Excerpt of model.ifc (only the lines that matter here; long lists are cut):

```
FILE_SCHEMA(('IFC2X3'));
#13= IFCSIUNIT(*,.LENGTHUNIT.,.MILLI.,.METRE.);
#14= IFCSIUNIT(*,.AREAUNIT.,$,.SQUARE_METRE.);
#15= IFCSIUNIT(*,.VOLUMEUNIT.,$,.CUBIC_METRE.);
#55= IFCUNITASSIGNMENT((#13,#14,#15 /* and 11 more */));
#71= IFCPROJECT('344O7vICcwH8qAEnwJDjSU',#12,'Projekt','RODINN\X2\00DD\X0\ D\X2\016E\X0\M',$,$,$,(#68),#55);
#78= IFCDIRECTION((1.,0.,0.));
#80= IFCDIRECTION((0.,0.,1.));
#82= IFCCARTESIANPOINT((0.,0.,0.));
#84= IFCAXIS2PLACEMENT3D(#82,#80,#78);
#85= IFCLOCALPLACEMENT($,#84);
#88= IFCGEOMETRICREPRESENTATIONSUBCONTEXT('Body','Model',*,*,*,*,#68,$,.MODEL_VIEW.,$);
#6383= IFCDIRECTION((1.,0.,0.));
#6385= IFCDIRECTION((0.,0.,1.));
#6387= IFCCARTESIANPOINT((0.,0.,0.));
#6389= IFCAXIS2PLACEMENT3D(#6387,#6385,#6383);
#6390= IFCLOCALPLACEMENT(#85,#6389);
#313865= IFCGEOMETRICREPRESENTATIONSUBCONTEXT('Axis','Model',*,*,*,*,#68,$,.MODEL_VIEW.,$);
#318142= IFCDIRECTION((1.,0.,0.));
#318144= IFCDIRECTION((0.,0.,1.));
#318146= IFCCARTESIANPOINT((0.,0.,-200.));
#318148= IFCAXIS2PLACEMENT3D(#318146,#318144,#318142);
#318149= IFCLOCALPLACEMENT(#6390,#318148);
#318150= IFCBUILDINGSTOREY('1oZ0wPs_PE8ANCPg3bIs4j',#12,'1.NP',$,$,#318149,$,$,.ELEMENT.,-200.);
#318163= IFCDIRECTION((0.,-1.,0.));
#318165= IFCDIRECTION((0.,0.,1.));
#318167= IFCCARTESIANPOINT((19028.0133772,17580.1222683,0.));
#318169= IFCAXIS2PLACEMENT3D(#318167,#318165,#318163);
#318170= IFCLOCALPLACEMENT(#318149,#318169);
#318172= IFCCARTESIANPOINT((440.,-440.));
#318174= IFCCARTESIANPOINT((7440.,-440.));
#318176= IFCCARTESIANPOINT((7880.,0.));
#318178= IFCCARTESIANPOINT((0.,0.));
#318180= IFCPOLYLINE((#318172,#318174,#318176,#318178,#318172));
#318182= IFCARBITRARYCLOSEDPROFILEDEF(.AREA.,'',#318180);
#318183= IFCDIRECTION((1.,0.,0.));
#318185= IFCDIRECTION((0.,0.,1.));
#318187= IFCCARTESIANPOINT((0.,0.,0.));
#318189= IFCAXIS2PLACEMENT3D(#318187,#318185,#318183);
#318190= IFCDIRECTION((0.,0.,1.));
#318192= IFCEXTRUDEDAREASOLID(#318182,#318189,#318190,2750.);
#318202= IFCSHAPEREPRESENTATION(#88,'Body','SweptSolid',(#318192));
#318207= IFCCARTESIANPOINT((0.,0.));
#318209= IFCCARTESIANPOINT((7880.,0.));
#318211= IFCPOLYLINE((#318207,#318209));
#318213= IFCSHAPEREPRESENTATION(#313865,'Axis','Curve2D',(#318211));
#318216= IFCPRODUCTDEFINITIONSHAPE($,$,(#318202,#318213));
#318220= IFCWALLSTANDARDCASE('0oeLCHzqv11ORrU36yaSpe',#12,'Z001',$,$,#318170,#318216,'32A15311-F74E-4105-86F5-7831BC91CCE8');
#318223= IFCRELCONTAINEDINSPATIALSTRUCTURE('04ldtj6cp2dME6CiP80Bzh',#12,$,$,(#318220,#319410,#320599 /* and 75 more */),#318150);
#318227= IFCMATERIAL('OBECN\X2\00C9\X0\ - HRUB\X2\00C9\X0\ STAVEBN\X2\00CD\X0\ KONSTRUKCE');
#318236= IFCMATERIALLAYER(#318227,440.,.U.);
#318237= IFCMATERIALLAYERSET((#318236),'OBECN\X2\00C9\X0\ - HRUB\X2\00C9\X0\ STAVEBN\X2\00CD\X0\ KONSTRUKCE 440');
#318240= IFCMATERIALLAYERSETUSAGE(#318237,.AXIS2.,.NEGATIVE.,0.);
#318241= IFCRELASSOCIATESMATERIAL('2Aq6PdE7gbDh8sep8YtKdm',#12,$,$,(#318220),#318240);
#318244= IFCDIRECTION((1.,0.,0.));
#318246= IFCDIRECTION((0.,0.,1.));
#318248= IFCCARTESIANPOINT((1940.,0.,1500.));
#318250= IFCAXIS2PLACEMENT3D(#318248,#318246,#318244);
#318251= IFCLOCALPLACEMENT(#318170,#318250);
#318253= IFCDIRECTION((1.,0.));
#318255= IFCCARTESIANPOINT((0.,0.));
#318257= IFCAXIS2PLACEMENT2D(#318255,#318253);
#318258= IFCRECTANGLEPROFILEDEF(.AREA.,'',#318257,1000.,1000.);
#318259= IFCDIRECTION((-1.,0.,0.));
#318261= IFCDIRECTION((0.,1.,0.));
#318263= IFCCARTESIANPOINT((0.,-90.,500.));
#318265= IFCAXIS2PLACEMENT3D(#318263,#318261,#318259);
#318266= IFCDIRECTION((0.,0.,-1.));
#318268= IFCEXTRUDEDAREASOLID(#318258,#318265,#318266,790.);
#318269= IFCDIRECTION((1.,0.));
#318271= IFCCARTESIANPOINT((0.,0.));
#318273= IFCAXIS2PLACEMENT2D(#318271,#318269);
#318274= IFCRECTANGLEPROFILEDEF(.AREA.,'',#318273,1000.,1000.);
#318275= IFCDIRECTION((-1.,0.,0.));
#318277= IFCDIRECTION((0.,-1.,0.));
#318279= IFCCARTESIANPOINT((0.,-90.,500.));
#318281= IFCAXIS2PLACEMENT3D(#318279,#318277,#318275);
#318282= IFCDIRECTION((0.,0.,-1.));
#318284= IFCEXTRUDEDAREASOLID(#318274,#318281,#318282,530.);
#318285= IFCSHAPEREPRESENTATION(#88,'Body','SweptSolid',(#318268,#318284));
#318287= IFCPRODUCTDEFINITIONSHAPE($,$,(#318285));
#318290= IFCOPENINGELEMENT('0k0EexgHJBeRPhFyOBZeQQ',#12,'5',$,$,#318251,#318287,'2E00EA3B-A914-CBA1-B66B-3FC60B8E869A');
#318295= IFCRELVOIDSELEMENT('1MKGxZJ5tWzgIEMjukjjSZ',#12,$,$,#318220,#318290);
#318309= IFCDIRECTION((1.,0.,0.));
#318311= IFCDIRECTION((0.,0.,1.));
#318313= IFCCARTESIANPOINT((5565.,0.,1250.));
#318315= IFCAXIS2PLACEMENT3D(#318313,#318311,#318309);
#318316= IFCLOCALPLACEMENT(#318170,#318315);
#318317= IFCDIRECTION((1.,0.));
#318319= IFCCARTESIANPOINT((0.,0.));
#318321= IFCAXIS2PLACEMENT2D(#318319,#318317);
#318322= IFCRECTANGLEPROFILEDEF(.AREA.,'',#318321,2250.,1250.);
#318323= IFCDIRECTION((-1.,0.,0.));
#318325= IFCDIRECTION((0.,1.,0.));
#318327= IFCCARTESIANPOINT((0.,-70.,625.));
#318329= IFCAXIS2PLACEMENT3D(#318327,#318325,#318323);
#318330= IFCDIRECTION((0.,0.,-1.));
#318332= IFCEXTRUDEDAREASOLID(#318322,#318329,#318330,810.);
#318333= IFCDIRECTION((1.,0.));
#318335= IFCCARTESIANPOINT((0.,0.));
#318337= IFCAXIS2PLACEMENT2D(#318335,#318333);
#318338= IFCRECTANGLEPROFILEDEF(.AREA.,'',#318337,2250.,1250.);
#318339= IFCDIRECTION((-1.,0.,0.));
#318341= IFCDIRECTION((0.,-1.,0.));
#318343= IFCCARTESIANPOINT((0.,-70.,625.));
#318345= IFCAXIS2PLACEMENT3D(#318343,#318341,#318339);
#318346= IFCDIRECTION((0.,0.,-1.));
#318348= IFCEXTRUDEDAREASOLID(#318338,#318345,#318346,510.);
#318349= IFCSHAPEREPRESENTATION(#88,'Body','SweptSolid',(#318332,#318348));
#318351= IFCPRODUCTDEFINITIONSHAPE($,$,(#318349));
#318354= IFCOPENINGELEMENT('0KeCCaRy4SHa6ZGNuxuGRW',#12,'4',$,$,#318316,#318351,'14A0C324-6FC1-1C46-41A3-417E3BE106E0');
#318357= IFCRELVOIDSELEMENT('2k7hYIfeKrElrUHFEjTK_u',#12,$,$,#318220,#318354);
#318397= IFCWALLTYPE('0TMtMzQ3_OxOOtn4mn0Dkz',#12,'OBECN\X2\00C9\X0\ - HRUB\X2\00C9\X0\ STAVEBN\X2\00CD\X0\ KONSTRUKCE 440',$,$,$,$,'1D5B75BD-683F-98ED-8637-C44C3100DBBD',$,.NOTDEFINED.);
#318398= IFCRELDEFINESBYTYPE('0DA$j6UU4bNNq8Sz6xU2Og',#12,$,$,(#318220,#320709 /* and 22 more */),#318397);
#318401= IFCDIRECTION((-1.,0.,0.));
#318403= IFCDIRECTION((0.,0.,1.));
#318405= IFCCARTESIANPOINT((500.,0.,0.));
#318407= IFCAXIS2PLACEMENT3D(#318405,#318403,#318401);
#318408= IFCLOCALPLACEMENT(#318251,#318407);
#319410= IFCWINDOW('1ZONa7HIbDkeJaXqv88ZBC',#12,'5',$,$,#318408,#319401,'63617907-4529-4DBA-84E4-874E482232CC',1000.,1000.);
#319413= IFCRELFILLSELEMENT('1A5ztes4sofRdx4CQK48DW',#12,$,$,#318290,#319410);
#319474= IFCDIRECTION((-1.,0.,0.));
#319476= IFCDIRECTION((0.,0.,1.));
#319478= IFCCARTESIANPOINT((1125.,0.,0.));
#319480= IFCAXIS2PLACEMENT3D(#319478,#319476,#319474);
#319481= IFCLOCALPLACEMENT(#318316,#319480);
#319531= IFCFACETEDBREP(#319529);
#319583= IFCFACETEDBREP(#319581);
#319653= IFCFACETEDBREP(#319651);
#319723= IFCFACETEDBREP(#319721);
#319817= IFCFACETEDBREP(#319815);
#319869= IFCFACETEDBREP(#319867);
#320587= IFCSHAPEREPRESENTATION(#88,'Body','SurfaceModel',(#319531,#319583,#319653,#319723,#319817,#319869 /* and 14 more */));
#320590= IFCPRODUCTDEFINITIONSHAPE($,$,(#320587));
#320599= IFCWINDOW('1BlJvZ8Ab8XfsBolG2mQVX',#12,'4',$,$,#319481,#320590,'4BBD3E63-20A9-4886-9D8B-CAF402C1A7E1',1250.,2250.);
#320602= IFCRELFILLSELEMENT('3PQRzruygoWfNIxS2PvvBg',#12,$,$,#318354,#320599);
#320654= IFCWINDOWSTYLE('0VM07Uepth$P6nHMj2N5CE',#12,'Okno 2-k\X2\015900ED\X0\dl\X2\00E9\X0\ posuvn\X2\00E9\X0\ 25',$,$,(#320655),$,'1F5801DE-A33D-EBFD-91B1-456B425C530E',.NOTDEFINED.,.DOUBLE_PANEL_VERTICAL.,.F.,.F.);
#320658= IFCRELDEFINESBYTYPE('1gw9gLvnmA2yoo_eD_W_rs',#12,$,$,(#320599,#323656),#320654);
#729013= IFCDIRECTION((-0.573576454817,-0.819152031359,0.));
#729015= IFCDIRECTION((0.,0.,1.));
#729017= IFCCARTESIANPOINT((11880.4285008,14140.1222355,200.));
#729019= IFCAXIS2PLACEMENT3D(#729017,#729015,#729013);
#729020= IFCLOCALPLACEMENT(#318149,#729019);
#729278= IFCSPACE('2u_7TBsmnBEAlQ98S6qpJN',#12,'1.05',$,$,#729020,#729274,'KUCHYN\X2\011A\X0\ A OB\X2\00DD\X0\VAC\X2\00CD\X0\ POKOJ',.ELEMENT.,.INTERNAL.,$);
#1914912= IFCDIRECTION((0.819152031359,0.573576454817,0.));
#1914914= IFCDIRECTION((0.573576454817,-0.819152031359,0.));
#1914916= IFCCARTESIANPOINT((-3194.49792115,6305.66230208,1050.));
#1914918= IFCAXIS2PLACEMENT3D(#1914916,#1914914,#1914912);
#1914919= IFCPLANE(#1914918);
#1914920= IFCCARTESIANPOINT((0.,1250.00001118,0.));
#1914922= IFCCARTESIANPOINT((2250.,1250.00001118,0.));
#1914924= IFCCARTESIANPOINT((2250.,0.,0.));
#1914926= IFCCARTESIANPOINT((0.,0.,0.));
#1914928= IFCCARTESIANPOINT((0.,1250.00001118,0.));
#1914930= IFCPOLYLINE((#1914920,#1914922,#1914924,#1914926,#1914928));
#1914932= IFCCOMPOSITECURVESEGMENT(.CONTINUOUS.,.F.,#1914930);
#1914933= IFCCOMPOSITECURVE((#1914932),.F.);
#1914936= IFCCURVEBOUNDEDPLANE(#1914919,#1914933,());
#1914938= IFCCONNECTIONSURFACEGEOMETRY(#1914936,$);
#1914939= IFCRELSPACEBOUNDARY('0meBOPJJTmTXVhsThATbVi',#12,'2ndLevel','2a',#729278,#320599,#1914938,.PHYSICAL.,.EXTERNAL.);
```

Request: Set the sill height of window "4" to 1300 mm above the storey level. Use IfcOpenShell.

```python
import numpy as np
import ifcopenshell
import ifcopenshell.api.geometry
import ifcopenshell.geom
import ifcopenshell.util.element
import ifcopenshell.util.placement
import ifcopenshell.util.shape
import ifcopenshell.util.unit

model = ifcopenshell.open("model.ifc")
unit_scale = ifcopenshell.util.unit.calculate_unit_scale(model)

window = model.by_guid("1BlJvZ8Ab8XfsBolG2mQVX")
opening = window.FillsVoids[0].RelatingOpeningElement
storey = ifcopenshell.util.element.get_container(window, ifc_class="IfcBuildingStorey")
level = ifcopenshell.util.placement.get_local_placement(storey.ObjectPlacement)[2, 3]

# The opening's origin need not be at the sill, so measure its lowest point.
shape = ifcopenshell.geom.create_shape(ifcopenshell.geom.settings(), opening)
bottom = ifcopenshell.util.shape.get_shape_bottom_elevation(shape, shape.geometry) / unit_scale
dz = level + 1.3 / unit_scale - bottom

shift = np.array([0.0, 0.0, dz])
# The window is placed relative to its opening, so it follows when the opening moves.
matrix = ifcopenshell.util.placement.get_local_placement(opening.ObjectPlacement)
matrix[:3, 3] += shift
ifcopenshell.api.geometry.edit_object_placement(
    model, product=opening, matrix=matrix, is_si=False, should_transform_children=True
)

# Space boundary surfaces are stored in each space's coordinates; move them too.
for rel in window.ProvidesBoundaries:
    if not rel.ConnectionGeometry:
        continue
    surface = rel.ConnectionGeometry.SurfaceOnRelatingElement.BasisSurface
    space_matrix = ifcopenshell.util.placement.get_local_placement(rel.RelatingSpace.ObjectPlacement)
    point = np.array(surface.Position.Location.Coordinates) + space_matrix[:3, :3].T @ shift
    surface.Position = model.createIfcAxis2Placement3D(
        model.createIfcCartesianPoint(point.tolist()), surface.Position.Axis, surface.Position.RefDirection
    )

print(f"moved by {dz * unit_scale:+.3f} m")

model.write("model_rev.ifc")
```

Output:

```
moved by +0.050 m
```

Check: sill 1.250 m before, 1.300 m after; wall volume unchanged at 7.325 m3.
